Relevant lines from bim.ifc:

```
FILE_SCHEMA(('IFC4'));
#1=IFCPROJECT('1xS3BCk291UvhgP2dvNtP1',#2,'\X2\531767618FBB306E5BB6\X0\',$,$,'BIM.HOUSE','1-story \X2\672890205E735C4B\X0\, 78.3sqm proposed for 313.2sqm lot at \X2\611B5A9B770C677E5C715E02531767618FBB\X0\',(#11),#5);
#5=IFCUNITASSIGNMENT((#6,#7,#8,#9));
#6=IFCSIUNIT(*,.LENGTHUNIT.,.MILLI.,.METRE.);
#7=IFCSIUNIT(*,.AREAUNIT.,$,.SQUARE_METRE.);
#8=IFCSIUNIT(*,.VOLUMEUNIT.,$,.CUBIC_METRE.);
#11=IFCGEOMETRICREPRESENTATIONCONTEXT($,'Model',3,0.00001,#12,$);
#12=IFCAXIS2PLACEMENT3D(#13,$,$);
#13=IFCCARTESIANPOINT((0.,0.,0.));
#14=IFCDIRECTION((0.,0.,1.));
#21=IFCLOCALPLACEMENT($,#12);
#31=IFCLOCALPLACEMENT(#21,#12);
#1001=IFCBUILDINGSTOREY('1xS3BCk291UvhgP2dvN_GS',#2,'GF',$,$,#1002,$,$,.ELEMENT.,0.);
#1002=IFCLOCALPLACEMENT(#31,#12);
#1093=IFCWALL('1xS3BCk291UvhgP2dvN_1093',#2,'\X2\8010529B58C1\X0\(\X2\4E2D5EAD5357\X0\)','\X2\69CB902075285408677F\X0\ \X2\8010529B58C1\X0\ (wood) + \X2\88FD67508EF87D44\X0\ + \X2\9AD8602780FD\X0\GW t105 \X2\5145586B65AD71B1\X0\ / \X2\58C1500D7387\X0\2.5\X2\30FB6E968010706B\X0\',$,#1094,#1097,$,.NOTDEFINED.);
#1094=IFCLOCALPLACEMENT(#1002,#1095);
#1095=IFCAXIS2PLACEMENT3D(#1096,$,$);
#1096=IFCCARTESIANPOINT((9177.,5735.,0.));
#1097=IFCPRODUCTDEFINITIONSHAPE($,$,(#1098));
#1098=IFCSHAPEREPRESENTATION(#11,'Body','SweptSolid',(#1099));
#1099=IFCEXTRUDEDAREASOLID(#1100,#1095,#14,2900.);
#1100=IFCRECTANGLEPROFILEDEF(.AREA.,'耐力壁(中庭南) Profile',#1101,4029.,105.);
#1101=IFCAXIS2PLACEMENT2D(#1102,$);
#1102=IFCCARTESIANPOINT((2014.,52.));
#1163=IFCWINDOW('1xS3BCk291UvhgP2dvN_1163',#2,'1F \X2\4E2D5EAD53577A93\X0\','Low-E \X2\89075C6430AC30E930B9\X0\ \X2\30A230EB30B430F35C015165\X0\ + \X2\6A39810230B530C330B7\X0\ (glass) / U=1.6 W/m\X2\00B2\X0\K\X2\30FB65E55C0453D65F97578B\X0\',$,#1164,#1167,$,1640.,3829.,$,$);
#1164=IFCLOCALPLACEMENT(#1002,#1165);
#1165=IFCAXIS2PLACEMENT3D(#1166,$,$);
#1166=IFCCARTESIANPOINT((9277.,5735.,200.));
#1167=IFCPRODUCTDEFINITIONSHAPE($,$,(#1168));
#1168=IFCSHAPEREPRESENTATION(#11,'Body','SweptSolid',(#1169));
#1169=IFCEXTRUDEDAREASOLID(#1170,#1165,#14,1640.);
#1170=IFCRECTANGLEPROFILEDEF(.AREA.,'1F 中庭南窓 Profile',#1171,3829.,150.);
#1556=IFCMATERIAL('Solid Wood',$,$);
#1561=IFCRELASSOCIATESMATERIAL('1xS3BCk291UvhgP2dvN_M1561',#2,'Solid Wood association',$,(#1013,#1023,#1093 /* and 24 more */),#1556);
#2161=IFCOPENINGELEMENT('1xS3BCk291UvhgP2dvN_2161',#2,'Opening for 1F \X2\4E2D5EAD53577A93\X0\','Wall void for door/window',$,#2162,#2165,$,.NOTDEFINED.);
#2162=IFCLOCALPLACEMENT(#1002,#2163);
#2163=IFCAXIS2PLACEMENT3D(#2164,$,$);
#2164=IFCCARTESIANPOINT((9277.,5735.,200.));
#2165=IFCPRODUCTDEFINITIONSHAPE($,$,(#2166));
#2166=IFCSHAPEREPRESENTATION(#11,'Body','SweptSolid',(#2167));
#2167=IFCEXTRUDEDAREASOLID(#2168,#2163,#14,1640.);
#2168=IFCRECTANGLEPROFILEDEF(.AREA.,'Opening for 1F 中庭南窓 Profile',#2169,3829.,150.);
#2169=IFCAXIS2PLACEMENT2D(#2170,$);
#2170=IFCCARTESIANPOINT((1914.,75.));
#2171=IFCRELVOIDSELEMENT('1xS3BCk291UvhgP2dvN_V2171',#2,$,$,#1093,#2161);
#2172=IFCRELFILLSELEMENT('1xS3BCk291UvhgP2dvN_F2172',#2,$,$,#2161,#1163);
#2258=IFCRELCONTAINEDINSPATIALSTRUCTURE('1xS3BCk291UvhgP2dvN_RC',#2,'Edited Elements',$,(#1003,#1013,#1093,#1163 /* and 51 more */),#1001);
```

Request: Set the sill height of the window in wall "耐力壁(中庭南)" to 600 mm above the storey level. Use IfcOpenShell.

```python
import numpy as np
import ifcopenshell
import ifcopenshell.api.geometry
import ifcopenshell.geom
import ifcopenshell.util.element
import ifcopenshell.util.placement
import ifcopenshell.util.shape
import ifcopenshell.util.unit

model = ifcopenshell.open("bim.ifc")
unit_scale = ifcopenshell.util.unit.calculate_unit_scale(model)

window = model.by_guid("1xS3BCk291UvhgP2dvN_1163")
opening = window.FillsVoids[0].RelatingOpeningElement
storey = ifcopenshell.util.element.get_container(window, ifc_class="IfcBuildingStorey")
level = ifcopenshell.util.placement.get_local_placement(storey.ObjectPlacement)[2, 3]

# The opening's origin need not be at the sill, so measure its lowest point.
shape = ifcopenshell.geom.create_shape(ifcopenshell.geom.settings(), opening)
bottom = ifcopenshell.util.shape.get_shape_bottom_elevation(shape, shape.geometry) / unit_scale
dz = level + 0.6 / unit_scale - bottom

shift = np.array([0.0, 0.0, dz])
# The window is not placed relative to its opening, so move both.
for product in (opening, window):
    matrix = ifcopenshell.util.placement.get_local_placement(product.ObjectPlacement)
    matrix[:3, 3] += shift
    ifcopenshell.api.geometry.edit_object_placement(model, product=product, matrix=matrix, is_si=False)

print(f"moved by {dz * unit_scale:+.3f} m")

model.write("bim-out.ifc")
```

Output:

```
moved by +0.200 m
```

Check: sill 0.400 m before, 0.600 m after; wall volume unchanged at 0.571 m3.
